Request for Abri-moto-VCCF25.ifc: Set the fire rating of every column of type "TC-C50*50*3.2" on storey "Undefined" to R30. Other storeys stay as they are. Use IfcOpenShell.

First a look at what the model holds.

```python
import ifcopenshell
import ifcopenshell.util.element

model = ifcopenshell.open("Abri-moto-VCCF25.ifc")
print(model.schema)
storey = next(s for s in model.by_type("IfcBuildingStorey") if s.Name == "Undefined")
columns = [e for e in ifcopenshell.util.element.get_decomposition(storey) if e.is_a("IfcColumn")]
seen = {}
for e in columns:
    element_type = ifcopenshell.util.element.get_type(e)
    key = (element_type.Name if element_type != e and element_type else None, ifcopenshell.util.element.get_pset(e, "Pset_ColumnCommon", "FireRating"))
    seen[key] = seen.get(key, 0) + 1
for (name, value), count in sorted(seen.items(), key=str):
    print(count, "x", name, "|", value)
```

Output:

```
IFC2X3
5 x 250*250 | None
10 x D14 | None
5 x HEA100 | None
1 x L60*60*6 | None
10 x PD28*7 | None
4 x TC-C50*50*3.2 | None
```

```python
import ifcopenshell
import ifcopenshell.api.pset
import ifcopenshell.util.element

model = ifcopenshell.open("Abri-moto-VCCF25.ifc")

storey = next(s for s in model.by_type("IfcBuildingStorey") if s.Name == "Undefined")
columns = [e for e in ifcopenshell.util.element.get_decomposition(storey) if e.is_a("IfcColumn")]

count = 0
for e in columns:
    element_type = ifcopenshell.util.element.get_type(e)
    if element_type in (None, e) or element_type.Name != "TC-C50*50*3.2":
        continue
    found = ifcopenshell.util.element.get_pset(e, "Pset_ColumnCommon", should_inherit=False)
    if found:
        pset = model.by_id(found["id"])
        if len(ifcopenshell.util.element.get_elements_by_pset(pset)) > 1:
            pset = ifcopenshell.api.pset.unshare_pset(model, products=[e], pset=pset)[0]
    else:
        pset = ifcopenshell.api.pset.add_pset(model, product=e, name="Pset_ColumnCommon")
    ifcopenshell.api.pset.edit_pset(model, pset=pset, properties={"FireRating": "R30"})
    count += 1

print(count, "columns updated")

model.write("Abri-moto-VCCF25-out.ifc")
```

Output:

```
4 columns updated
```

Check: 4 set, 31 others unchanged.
